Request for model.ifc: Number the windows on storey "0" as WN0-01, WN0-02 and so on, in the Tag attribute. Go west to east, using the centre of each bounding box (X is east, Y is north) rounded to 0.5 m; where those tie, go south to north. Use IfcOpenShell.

First a look at what the model holds.

```python
import ifcopenshell
import ifcopenshell.util.element
import ifcopenshell.util.placement

model = ifcopenshell.open("model.ifc")
print(model.schema)
storey = next(s for s in model.by_type("IfcBuildingStorey") if s.Name == "0")
windows = [e for e in ifcopenshell.util.element.get_decomposition(storey) if e.is_a("IfcWindow")]
for e in sorted(windows, key=lambda e: e.id()):
    origin = ifcopenshell.util.placement.get_local_placement(e.ObjectPlacement)[:3, 3]
    print(e.id(), e.Tag, e.Name, origin.round(2) + 0.0, sep=" | ")
```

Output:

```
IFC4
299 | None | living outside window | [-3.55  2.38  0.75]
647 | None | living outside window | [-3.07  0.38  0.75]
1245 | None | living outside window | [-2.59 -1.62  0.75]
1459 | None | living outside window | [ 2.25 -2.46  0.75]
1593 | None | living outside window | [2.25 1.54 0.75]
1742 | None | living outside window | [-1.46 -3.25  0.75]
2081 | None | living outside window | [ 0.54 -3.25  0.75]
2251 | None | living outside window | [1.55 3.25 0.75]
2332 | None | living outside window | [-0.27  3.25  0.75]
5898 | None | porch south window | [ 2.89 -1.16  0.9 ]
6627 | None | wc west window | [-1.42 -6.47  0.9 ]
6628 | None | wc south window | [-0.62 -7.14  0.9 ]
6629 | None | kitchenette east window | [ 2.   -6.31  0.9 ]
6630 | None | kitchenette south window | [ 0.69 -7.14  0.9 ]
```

```python
import ifcopenshell
import ifcopenshell.geom
import ifcopenshell.util.element
import ifcopenshell.util.shape

model = ifcopenshell.open("model.ifc")
settings = ifcopenshell.geom.settings()
settings.set("use-world-coords", True)


def centre(element):
    shape = ifcopenshell.geom.create_shape(settings, element)
    return ifcopenshell.util.shape.get_bbox_centroid(shape.geometry)


storey = next(s for s in model.by_type("IfcBuildingStorey") if s.Name == "0")
windows = [e for e in ifcopenshell.util.element.get_decomposition(storey) if e.is_a("IfcWindow")]

# Insertion points can sit at a corner or the storey origin, so sort by the geometry (in metres).
centres = {e: centre(e) for e in windows}
windows.sort(key=lambda e: (round(centres[e][0] / 0.5), centres[e][1]))

for i, e in enumerate(windows, start=1):
    number = f"WN0-{i:02d}"
    e.Tag = number
    print(e.id(), number)

model.write("model-out.ifc")
```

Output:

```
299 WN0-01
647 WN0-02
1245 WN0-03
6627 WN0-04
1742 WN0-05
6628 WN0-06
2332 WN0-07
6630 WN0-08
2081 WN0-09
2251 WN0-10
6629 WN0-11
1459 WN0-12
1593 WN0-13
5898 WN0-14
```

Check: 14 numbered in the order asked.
